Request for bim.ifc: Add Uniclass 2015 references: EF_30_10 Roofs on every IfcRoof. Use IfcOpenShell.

First a look at what the model holds.

```python
import ifcopenshell

model = ifcopenshell.open("bim.ifc")
print(model.schema)
print("classifications:", [c.Name for c in model.by_type("IfcClassification")])
for ifc_class in ("IfcDoor", "IfcRoof", "IfcStair", "IfcWall", "IfcWindow"):
    print(ifc_class, len(model.by_type(ifc_class)))
```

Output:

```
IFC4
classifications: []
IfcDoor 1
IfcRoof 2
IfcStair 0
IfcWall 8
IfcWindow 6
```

```python
import ifcopenshell
import ifcopenshell.api.classification

model = ifcopenshell.open("bim.ifc")

system = ifcopenshell.api.classification.add_classification(model, classification="Uniclass 2015")

codes = {
    "IfcRoof": ("EF_30_10", "Roofs"),
}
for ifc_class, (code, name) in codes.items():
    products = model.by_type(ifc_class)
    ifcopenshell.api.classification.add_reference(
        model, products=products, classification=system, identification=code, name=name
    )
    print(code, len(products))

model.write("bim-out.ifc")
```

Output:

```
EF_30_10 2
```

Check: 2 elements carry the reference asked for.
